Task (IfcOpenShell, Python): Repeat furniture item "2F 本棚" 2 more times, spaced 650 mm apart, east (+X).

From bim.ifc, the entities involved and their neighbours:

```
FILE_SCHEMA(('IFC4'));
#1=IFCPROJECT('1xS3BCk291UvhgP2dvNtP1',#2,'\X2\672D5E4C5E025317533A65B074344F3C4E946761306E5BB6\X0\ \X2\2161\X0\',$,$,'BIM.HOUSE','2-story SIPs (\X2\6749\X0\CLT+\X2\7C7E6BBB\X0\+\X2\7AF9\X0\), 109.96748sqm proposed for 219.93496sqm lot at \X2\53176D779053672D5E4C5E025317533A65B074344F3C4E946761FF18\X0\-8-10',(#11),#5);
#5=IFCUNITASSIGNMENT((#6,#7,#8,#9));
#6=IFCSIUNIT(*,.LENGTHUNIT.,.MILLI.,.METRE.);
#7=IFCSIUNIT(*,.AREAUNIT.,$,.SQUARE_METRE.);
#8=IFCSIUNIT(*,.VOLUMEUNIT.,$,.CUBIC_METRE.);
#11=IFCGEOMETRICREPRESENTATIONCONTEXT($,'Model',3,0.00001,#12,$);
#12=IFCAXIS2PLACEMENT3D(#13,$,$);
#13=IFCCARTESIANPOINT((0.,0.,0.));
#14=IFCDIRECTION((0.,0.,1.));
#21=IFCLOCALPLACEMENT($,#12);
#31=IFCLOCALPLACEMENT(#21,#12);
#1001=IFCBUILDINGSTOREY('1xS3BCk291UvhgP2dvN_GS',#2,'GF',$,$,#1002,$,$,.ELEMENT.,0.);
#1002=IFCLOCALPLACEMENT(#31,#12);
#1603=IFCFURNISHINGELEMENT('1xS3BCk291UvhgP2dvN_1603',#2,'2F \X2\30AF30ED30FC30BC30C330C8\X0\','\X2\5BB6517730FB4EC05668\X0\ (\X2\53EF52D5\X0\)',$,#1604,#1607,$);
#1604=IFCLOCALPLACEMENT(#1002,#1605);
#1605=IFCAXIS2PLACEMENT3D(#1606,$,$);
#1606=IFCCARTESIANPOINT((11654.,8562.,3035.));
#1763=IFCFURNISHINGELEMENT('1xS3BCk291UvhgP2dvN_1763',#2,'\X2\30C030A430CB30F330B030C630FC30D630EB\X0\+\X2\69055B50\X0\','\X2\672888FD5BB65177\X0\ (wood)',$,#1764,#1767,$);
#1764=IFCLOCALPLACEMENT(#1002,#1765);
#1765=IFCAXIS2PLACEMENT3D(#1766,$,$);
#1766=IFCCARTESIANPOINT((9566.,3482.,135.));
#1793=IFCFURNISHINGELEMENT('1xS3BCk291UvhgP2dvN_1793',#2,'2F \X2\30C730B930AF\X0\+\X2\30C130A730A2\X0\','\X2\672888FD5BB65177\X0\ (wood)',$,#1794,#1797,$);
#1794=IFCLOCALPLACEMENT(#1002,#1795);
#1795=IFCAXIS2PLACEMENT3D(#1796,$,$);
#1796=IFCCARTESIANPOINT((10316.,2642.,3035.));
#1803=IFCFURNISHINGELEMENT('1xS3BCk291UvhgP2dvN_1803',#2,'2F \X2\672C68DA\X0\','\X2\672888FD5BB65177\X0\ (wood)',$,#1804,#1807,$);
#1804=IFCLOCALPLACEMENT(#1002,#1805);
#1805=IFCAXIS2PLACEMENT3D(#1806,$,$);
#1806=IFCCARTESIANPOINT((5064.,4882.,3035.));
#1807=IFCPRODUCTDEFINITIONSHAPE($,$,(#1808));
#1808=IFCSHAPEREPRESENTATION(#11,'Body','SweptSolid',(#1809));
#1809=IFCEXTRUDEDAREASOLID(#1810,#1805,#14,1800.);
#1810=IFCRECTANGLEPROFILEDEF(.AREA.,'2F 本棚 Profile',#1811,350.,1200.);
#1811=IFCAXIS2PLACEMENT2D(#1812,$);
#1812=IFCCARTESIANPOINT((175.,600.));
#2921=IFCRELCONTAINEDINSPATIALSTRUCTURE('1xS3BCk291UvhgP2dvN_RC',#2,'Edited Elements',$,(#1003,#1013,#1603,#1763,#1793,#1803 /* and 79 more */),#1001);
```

```python
import numpy as np
import ifcopenshell
import ifcopenshell.api.geometry
import ifcopenshell.api.root
import ifcopenshell.util.element
import ifcopenshell.util.placement
import ifcopenshell.util.unit

model = ifcopenshell.open("bim.ifc")
unit_scale = ifcopenshell.util.unit.calculate_unit_scale(model)


def reuse_history(source, copy):
    """copy_class also copies each property set's owner history, people and application; keep the originals."""
    for rel in copy.IsDefinedBy:
        if rel.is_a("IfcRelDefinesByProperties") and (history := rel.RelatingPropertyDefinition.OwnerHistory):
            rel.RelatingPropertyDefinition.OwnerHistory = source.OwnerHistory
            ifcopenshell.util.element.remove_deep2(model, history)


source = model.by_guid("1xS3BCk291UvhgP2dvN_1803")
base = ifcopenshell.util.placement.get_local_placement(source.ObjectPlacement)
step = np.array([1.0, 0.0, 0.0]) * 0.65 / unit_scale

for i in range(1, 3):
    copy = ifcopenshell.api.root.copy_class(model, product=source)
    copy.Representation = ifcopenshell.util.element.copy_deep(
        model, source.Representation, exclude=["IfcGeometricRepresentationContext", "IfcRepresentationMap"]
    )
    reuse_history(source, copy)
    matrix = base.copy()
    matrix[:3, 3] += i * step
    print("added at", matrix[:3, 3].round(3) + 0.0)
    ifcopenshell.api.geometry.edit_object_placement(model, product=copy, matrix=matrix, is_si=False)

model.write("bim-out.ifc")
```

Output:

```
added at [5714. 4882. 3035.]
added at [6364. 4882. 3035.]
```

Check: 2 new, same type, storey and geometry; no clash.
